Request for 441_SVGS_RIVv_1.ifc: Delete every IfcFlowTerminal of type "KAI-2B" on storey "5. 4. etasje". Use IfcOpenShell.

First a look at what the model holds.

```python
import ifcopenshell
import ifcopenshell.util.element

model = ifcopenshell.open("441_SVGS_RIVv_1.ifc")
print(model.schema)
storey = next(s for s in model.by_type("IfcBuildingStorey") if s.Name == "5. 4. etasje")
terminals = [e for e in ifcopenshell.util.element.get_decomposition(storey) if e.is_a("IfcFlowTerminal")]
seen = {}
for e in terminals:
    element_type = ifcopenshell.util.element.get_type(e)
    name = element_type.Name if element_type not in (None, e) else None
    seen[name] = seen.get(name, 0) + 1
for name, count in sorted(seen.items(), key=str):
    print(count, "x", name)
```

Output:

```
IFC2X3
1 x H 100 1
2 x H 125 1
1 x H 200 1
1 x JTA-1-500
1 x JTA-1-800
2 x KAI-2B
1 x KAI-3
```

```python
import ifcopenshell
import ifcopenshell.api.root
import ifcopenshell.util.element

model = ifcopenshell.open("441_SVGS_RIVv_1.ifc")

storey = next(s for s in model.by_type("IfcBuildingStorey") if s.Name == "5. 4. etasje")
terminals = [e for e in ifcopenshell.util.element.get_decomposition(storey) if e.is_a("IfcFlowTerminal")]
targets = [e for e in terminals if (t := ifcopenshell.util.element.get_type(e)) not in (None, e) and t.Name == "KAI-2B"]

for e in targets:
    ifcopenshell.api.root.remove_product(model, product=e)
print(len(targets), "removed")

model.write("441_SVGS_RIVv_1_edited.ifc")
```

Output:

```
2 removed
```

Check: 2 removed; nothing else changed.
